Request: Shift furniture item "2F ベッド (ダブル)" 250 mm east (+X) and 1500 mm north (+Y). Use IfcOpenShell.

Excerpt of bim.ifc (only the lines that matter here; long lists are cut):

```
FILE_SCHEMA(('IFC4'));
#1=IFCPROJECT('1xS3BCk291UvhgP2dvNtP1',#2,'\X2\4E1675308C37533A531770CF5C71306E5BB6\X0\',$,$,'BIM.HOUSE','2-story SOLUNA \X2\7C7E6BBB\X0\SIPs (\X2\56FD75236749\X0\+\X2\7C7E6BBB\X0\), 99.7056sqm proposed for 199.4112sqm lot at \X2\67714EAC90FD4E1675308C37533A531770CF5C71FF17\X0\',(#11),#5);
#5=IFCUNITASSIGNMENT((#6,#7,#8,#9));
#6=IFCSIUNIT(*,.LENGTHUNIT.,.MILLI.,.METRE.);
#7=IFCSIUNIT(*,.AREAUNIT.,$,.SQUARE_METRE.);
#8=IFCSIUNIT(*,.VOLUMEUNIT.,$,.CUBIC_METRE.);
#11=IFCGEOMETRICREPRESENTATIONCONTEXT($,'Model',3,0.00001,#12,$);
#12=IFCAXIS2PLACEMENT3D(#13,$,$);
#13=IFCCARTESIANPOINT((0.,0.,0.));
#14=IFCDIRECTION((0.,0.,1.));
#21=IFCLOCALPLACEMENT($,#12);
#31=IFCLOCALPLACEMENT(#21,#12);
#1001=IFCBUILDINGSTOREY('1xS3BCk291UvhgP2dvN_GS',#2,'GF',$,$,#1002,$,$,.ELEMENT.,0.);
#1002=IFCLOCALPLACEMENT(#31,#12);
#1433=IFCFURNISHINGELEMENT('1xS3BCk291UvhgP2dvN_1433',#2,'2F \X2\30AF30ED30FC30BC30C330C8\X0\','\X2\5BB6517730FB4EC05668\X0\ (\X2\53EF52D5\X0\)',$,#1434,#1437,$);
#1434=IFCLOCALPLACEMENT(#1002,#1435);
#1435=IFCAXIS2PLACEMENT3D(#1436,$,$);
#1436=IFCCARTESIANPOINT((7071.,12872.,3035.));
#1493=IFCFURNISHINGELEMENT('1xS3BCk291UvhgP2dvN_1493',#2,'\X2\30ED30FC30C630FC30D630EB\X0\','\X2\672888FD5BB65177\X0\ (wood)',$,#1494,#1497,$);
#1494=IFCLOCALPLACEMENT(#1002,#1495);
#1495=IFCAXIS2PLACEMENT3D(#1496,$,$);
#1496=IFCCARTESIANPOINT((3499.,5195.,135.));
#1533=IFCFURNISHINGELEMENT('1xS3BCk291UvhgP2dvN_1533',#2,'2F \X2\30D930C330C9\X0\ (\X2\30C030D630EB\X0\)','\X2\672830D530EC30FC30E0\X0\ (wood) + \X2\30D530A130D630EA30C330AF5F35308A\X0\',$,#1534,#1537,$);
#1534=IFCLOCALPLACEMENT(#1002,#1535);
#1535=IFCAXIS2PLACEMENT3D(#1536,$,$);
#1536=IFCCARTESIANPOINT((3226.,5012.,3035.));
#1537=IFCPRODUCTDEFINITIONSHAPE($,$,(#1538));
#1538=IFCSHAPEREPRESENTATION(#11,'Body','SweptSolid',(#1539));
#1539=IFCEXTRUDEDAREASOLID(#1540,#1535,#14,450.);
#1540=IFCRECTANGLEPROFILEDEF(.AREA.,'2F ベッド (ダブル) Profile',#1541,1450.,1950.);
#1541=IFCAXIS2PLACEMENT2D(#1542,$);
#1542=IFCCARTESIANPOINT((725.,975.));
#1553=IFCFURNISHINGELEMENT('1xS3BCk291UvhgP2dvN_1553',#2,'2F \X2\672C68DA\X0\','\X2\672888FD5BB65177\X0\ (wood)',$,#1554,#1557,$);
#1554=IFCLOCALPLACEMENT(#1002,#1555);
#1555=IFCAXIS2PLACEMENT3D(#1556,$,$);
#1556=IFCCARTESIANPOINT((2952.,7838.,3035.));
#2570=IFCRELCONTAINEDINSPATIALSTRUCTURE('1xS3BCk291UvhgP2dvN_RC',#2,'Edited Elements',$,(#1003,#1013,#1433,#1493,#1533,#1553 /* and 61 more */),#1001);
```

```python
import ifcopenshell
import ifcopenshell.api.geometry
import ifcopenshell.util.placement
import ifcopenshell.util.unit

model = ifcopenshell.open("bim.ifc")
unit_scale = ifcopenshell.util.unit.calculate_unit_scale(model)

item = model.by_guid("1xS3BCk291UvhgP2dvN_1533")
matrix = ifcopenshell.util.placement.get_local_placement(item.ObjectPlacement)
matrix[0, 3] += 0.25 / unit_scale
matrix[1, 3] += 1.5 / unit_scale
ifcopenshell.api.geometry.edit_object_placement(model, product=item, matrix=matrix, is_si=False)

print(ifcopenshell.util.placement.get_local_placement(item.ObjectPlacement).round(3) + 0.0)

model.write("bim_rev.ifc")
```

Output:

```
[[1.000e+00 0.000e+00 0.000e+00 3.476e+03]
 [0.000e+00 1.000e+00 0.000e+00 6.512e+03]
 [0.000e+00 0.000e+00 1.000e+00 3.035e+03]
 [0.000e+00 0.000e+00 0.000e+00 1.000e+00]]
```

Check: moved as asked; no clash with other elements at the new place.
